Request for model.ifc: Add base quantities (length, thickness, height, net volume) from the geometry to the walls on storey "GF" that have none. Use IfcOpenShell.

First a look at what the model holds.

```python
import ifcopenshell
import ifcopenshell.util.element
import ifcopenshell.util.unit

model = ifcopenshell.open("model.ifc")
print(model.schema)
for unit_type in ("LENGTHUNIT", "AREAUNIT", "VOLUMEUNIT"):
    print(unit_type, ifcopenshell.util.unit.calculate_unit_scale(model, unit_type))
storey = next(s for s in model.by_type("IfcBuildingStorey") if s.Name == "GF")
walls = [e for e in ifcopenshell.util.element.get_decomposition(storey) if e.is_a("IfcWall")]
for e in sorted(walls, key=lambda e: e.id()):
    print(e.id(), e.is_a(), e.Name, list(ifcopenshell.util.element.get_psets(e, qtos_only=True)), sep=" | ")
```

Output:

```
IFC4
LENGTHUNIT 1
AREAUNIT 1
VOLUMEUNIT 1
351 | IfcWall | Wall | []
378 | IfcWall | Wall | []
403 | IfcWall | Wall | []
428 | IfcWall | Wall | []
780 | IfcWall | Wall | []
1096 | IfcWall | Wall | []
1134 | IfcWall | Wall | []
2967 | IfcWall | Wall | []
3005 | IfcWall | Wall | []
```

```python
import ifcopenshell
import ifcopenshell.api.pset
import ifcopenshell.geom
import ifcopenshell.util.element
import ifcopenshell.util.shape
import ifcopenshell.util.unit

model = ifcopenshell.open("model.ifc")
unit_scale = ifcopenshell.util.unit.calculate_unit_scale(model)
volume_scale = ifcopenshell.util.unit.calculate_unit_scale(model, "VOLUMEUNIT")
settings = ifcopenshell.geom.settings()

storey = next(s for s in model.by_type("IfcBuildingStorey") if s.Name == "GF")
walls = [e for e in ifcopenshell.util.element.get_decomposition(storey) if e.is_a("IfcWall")]

for e in sorted(walls, key=lambda e: e.id()):
    if ifcopenshell.util.element.get_psets(e, qtos_only=True, should_inherit=False):
        continue
    # Geometry comes back in metres, in the element's own axes.
    shape = ifcopenshell.geom.create_shape(settings, e)
    values = {
        "Length": ifcopenshell.util.shape.get_x(shape.geometry) / unit_scale,
        "Width": ifcopenshell.util.shape.get_y(shape.geometry) / unit_scale,
        "Height": ifcopenshell.util.shape.get_z(shape.geometry) / unit_scale,
        "NetVolume": ifcopenshell.util.shape.get_volume(shape.geometry) / volume_scale,
    }
    qto = ifcopenshell.api.pset.add_qto(model, product=e, name="Qto_WallBaseQuantities")
    ifcopenshell.api.pset.edit_qto(model, qto=qto, properties=values)
    print(e.id(), {k: round(v, 3) for k, v in values.items()})

model.write("model_rev.ifc")
```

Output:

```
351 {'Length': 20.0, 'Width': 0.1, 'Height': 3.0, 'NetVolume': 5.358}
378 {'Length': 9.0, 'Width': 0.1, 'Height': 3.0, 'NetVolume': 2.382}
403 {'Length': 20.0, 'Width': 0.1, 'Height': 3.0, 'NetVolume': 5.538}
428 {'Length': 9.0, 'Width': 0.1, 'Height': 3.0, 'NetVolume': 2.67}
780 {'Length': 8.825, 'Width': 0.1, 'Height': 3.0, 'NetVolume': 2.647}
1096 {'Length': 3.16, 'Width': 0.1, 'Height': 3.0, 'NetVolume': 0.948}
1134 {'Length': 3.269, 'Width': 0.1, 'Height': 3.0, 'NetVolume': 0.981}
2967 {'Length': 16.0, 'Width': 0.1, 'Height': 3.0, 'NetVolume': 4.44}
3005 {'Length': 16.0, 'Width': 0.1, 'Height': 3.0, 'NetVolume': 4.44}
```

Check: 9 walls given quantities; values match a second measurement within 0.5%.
